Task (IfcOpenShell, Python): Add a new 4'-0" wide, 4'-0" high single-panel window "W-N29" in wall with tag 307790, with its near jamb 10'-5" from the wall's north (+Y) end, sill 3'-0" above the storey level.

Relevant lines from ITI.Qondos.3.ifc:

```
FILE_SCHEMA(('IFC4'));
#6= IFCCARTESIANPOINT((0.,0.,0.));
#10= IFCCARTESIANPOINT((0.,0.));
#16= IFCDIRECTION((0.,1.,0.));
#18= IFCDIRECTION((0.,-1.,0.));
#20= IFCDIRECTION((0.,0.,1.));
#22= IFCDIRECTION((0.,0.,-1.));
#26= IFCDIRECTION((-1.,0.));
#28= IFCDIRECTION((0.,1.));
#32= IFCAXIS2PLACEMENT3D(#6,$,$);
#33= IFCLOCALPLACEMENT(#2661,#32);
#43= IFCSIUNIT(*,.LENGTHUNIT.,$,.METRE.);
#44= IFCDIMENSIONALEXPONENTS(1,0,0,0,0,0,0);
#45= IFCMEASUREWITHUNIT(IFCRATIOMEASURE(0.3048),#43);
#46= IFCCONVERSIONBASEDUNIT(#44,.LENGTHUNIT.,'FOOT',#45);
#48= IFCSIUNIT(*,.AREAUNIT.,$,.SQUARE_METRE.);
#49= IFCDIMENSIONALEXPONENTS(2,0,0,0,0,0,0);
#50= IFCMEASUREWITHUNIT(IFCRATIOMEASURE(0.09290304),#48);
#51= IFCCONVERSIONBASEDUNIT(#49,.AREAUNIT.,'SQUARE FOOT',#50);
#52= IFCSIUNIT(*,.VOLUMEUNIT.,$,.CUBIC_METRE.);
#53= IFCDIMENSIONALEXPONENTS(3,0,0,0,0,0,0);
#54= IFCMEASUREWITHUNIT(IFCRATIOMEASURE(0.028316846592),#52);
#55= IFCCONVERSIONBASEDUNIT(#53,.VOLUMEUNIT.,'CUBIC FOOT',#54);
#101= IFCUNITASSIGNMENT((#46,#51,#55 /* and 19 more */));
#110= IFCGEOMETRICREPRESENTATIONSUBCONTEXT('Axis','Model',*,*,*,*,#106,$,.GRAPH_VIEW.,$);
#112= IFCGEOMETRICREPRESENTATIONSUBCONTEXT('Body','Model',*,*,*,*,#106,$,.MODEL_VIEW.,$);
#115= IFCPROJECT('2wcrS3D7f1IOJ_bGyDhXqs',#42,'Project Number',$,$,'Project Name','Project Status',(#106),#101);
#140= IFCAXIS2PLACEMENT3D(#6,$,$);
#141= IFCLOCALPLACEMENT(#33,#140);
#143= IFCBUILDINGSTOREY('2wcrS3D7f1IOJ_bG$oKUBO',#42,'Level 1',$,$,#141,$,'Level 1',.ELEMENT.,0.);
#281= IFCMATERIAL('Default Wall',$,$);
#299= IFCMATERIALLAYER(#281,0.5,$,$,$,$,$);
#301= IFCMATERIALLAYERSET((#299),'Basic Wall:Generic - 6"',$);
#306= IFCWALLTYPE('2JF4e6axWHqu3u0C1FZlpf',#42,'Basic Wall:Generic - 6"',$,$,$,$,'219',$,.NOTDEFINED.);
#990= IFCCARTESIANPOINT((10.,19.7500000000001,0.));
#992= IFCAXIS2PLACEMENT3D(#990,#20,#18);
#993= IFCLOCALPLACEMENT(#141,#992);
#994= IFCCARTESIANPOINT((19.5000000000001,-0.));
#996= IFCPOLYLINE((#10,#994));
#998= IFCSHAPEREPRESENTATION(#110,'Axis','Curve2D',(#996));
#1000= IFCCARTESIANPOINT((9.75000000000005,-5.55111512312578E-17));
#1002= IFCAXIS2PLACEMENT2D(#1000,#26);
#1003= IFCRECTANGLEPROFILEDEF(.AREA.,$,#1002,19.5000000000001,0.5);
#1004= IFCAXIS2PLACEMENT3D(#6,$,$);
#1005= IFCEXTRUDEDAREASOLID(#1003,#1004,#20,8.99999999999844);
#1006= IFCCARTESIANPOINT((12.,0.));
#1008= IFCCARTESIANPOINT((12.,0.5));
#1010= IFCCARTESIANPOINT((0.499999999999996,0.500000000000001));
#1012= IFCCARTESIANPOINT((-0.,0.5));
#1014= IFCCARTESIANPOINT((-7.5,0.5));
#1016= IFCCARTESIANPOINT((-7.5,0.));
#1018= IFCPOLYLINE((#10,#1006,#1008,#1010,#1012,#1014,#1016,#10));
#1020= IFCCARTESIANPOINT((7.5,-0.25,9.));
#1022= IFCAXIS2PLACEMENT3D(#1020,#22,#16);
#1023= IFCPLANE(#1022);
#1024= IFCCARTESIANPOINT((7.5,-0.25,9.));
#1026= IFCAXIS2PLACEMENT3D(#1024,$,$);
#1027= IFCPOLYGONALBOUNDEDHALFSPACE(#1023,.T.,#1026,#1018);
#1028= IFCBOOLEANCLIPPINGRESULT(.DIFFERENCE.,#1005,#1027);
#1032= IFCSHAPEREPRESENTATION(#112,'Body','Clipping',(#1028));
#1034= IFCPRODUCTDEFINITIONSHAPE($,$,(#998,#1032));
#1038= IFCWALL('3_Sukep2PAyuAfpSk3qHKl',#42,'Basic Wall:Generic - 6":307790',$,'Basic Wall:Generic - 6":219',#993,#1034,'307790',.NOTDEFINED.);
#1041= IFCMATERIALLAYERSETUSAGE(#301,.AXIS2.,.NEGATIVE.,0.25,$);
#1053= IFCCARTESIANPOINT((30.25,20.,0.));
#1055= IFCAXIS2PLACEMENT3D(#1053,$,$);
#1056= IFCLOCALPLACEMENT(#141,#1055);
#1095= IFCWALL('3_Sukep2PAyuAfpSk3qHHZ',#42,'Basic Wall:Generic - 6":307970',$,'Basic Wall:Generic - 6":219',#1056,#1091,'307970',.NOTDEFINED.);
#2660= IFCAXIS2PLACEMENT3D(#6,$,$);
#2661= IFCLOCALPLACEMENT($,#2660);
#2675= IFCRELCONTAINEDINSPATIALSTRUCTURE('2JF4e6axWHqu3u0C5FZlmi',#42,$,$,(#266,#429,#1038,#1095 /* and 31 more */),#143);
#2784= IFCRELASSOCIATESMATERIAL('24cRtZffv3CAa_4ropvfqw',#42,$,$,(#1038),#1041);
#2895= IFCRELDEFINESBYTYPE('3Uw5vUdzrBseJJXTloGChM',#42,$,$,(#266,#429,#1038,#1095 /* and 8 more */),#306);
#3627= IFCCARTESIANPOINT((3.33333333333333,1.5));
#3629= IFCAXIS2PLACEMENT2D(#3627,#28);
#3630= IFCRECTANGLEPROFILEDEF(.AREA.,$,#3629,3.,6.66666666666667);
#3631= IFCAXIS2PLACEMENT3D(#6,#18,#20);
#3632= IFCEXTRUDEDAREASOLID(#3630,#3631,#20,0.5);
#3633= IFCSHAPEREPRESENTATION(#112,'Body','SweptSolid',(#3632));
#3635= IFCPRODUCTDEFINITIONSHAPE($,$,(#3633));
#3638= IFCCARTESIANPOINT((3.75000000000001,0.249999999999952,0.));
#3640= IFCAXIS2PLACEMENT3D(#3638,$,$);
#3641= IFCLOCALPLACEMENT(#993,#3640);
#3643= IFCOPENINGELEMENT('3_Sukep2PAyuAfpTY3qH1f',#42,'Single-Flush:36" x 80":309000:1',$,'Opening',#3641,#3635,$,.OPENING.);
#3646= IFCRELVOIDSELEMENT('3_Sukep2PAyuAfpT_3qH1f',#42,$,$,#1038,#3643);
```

```python
import numpy as np
import ifcopenshell
import ifcopenshell.api.feature
import ifcopenshell.api.geometry
import ifcopenshell.api.root
import ifcopenshell.api.spatial
import ifcopenshell.geom
import ifcopenshell.util.element
import ifcopenshell.util.placement
import ifcopenshell.util.representation
import ifcopenshell.util.shape
import ifcopenshell.util.unit

model = ifcopenshell.open("ITI.Qondos.3.ifc")
unit_scale = ifcopenshell.util.unit.calculate_unit_scale(model)
settings = ifcopenshell.geom.settings()


def volume(element):
    """Net volume in cubic metres, openings subtracted."""
    shape = ifcopenshell.geom.create_shape(settings, element)
    return ifcopenshell.util.shape.get_volume(shape.geometry)


wall = model.by_guid("3_Sukep2PAyuAfpSk3qHKl")
storey = ifcopenshell.util.element.get_container(wall, ifc_class="IfcBuildingStorey")
context = ifcopenshell.util.representation.get_context(model, "Model", "Body", "MODEL_VIEW")
before = volume(wall)

width, height, from_end, sill = 1.2192, 1.2192, 3.175, 0.9144  # metres

# The wall runs along its own X axis, and the end named is its -X end.
wall_shape = ifcopenshell.geom.create_shape(settings, wall)
x, y, z = ifcopenshell.util.shape.get_vertices(wall_shape.geometry).T
start = x.min() + from_end
face, thickness = float(y.min()), float(y.max() - y.min())
wall_matrix = ifcopenshell.util.placement.get_local_placement(wall.ObjectPlacement)
level = ifcopenshell.util.placement.get_local_placement(storey.ObjectPlacement)[2, 3]


def in_wall(x, y):
    """Placement at x, y metres in the wall's axes, at sill height."""
    matrix = wall_matrix.copy()
    matrix[:, 3] = wall_matrix @ np.array([x / unit_scale, y / unit_scale, 0.0, 1.0])
    matrix[2, 3] = level + sill / unit_scale
    return matrix


# Opening: a box that overshoots both wall faces by 50 mm.
opening = ifcopenshell.api.root.create_entity(model, ifc_class="IfcOpeningElement", predefined_type="OPENING")
box = ifcopenshell.api.geometry.add_wall_representation(
    model, context=context, length=width, height=height, thickness=thickness + 0.1
)
ifcopenshell.api.geometry.assign_representation(model, product=opening, representation=box)
ifcopenshell.api.geometry.edit_object_placement(model, product=opening, matrix=in_wall(start, face - 0.05), is_si=False)
ifcopenshell.api.feature.add_feature(model, feature=opening, element=wall)

window = ifcopenshell.api.root.create_entity(model, ifc_class="IfcWindow", name="W-N29", predefined_type="WINDOW")
window.OverallWidth, window.OverallHeight = width / unit_scale, height / unit_scale
window.PartitioningType = "SINGLE_PANEL"
body = ifcopenshell.api.geometry.add_window_representation(
    model,
    context=context,
    overall_width=window.OverallWidth,
    overall_height=window.OverallHeight,
    partition_type="SINGLE_PANEL",
)
ifcopenshell.api.geometry.assign_representation(model, product=window, representation=body)
ifcopenshell.api.spatial.assign_container(model, products=[window], relating_structure=storey)
ifcopenshell.api.feature.add_filling(model, opening=opening, element=window)

# Centre the window in the wall's thickness.
ifcopenshell.api.geometry.edit_object_placement(model, product=window, matrix=in_wall(start, face), is_si=False)
window_shape = ifcopenshell.geom.create_shape(settings, window)
depth = ifcopenshell.util.shape.get_vertices(window_shape.geometry)[:, 1]
offset = face + thickness / 2 - (depth.min() + depth.max()) / 2
ifcopenshell.api.geometry.edit_object_placement(model, product=window, matrix=in_wall(start, offset), is_si=False)

after = volume(wall)

print(f"wall volume {before:.3f} -> {after:.3f} m3")

model.write("ITI.Qondos.3_updated.ifc")
```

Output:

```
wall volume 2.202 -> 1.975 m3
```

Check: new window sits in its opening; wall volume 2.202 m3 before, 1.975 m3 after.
